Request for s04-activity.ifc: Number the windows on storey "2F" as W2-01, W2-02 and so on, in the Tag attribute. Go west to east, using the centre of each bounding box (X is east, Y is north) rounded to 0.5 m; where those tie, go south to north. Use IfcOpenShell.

First a look at what the model holds.

```python
import ifcopenshell
import ifcopenshell.util.element
import ifcopenshell.util.placement

model = ifcopenshell.open("s04-activity.ifc")
print(model.schema)
storey = next(s for s in model.by_type("IfcBuildingStorey") if s.Name == "2F")
windows = [e for e in ifcopenshell.util.element.get_decomposition(storey) if e.is_a("IfcWindow")]
for e in sorted(windows, key=lambda e: e.id()):
    origin = ifcopenshell.util.placement.get_local_placement(e.ObjectPlacement)[:3, 3]
    print(e.id(), e.Tag, e.Name, origin.round(2) + 0.0, sep=" | ")
```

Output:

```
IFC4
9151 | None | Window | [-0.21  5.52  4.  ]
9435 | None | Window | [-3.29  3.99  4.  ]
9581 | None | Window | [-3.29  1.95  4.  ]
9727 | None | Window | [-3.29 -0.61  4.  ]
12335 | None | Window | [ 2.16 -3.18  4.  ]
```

```python
import ifcopenshell
import ifcopenshell.geom
import ifcopenshell.util.element
import ifcopenshell.util.shape

model = ifcopenshell.open("s04-activity.ifc")
settings = ifcopenshell.geom.settings()
settings.set("use-world-coords", True)


def centre(element):
    shape = ifcopenshell.geom.create_shape(settings, element)
    return ifcopenshell.util.shape.get_bbox_centroid(shape.geometry)


storey = next(s for s in model.by_type("IfcBuildingStorey") if s.Name == "2F")
windows = [e for e in ifcopenshell.util.element.get_decomposition(storey) if e.is_a("IfcWindow")]

# Insertion points can sit at a corner or the storey origin, so sort by the geometry (in metres).
centres = {e: centre(e) for e in windows}
windows.sort(key=lambda e: (round(centres[e][0] / 0.5), centres[e][1]))

for i, e in enumerate(windows, start=1):
    number = f"W2-{i:02d}"
    e.Tag = number
    print(e.id(), number)

model.write("s04-activity_rev.ifc")
```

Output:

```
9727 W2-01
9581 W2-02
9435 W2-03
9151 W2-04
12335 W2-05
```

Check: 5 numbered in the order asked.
